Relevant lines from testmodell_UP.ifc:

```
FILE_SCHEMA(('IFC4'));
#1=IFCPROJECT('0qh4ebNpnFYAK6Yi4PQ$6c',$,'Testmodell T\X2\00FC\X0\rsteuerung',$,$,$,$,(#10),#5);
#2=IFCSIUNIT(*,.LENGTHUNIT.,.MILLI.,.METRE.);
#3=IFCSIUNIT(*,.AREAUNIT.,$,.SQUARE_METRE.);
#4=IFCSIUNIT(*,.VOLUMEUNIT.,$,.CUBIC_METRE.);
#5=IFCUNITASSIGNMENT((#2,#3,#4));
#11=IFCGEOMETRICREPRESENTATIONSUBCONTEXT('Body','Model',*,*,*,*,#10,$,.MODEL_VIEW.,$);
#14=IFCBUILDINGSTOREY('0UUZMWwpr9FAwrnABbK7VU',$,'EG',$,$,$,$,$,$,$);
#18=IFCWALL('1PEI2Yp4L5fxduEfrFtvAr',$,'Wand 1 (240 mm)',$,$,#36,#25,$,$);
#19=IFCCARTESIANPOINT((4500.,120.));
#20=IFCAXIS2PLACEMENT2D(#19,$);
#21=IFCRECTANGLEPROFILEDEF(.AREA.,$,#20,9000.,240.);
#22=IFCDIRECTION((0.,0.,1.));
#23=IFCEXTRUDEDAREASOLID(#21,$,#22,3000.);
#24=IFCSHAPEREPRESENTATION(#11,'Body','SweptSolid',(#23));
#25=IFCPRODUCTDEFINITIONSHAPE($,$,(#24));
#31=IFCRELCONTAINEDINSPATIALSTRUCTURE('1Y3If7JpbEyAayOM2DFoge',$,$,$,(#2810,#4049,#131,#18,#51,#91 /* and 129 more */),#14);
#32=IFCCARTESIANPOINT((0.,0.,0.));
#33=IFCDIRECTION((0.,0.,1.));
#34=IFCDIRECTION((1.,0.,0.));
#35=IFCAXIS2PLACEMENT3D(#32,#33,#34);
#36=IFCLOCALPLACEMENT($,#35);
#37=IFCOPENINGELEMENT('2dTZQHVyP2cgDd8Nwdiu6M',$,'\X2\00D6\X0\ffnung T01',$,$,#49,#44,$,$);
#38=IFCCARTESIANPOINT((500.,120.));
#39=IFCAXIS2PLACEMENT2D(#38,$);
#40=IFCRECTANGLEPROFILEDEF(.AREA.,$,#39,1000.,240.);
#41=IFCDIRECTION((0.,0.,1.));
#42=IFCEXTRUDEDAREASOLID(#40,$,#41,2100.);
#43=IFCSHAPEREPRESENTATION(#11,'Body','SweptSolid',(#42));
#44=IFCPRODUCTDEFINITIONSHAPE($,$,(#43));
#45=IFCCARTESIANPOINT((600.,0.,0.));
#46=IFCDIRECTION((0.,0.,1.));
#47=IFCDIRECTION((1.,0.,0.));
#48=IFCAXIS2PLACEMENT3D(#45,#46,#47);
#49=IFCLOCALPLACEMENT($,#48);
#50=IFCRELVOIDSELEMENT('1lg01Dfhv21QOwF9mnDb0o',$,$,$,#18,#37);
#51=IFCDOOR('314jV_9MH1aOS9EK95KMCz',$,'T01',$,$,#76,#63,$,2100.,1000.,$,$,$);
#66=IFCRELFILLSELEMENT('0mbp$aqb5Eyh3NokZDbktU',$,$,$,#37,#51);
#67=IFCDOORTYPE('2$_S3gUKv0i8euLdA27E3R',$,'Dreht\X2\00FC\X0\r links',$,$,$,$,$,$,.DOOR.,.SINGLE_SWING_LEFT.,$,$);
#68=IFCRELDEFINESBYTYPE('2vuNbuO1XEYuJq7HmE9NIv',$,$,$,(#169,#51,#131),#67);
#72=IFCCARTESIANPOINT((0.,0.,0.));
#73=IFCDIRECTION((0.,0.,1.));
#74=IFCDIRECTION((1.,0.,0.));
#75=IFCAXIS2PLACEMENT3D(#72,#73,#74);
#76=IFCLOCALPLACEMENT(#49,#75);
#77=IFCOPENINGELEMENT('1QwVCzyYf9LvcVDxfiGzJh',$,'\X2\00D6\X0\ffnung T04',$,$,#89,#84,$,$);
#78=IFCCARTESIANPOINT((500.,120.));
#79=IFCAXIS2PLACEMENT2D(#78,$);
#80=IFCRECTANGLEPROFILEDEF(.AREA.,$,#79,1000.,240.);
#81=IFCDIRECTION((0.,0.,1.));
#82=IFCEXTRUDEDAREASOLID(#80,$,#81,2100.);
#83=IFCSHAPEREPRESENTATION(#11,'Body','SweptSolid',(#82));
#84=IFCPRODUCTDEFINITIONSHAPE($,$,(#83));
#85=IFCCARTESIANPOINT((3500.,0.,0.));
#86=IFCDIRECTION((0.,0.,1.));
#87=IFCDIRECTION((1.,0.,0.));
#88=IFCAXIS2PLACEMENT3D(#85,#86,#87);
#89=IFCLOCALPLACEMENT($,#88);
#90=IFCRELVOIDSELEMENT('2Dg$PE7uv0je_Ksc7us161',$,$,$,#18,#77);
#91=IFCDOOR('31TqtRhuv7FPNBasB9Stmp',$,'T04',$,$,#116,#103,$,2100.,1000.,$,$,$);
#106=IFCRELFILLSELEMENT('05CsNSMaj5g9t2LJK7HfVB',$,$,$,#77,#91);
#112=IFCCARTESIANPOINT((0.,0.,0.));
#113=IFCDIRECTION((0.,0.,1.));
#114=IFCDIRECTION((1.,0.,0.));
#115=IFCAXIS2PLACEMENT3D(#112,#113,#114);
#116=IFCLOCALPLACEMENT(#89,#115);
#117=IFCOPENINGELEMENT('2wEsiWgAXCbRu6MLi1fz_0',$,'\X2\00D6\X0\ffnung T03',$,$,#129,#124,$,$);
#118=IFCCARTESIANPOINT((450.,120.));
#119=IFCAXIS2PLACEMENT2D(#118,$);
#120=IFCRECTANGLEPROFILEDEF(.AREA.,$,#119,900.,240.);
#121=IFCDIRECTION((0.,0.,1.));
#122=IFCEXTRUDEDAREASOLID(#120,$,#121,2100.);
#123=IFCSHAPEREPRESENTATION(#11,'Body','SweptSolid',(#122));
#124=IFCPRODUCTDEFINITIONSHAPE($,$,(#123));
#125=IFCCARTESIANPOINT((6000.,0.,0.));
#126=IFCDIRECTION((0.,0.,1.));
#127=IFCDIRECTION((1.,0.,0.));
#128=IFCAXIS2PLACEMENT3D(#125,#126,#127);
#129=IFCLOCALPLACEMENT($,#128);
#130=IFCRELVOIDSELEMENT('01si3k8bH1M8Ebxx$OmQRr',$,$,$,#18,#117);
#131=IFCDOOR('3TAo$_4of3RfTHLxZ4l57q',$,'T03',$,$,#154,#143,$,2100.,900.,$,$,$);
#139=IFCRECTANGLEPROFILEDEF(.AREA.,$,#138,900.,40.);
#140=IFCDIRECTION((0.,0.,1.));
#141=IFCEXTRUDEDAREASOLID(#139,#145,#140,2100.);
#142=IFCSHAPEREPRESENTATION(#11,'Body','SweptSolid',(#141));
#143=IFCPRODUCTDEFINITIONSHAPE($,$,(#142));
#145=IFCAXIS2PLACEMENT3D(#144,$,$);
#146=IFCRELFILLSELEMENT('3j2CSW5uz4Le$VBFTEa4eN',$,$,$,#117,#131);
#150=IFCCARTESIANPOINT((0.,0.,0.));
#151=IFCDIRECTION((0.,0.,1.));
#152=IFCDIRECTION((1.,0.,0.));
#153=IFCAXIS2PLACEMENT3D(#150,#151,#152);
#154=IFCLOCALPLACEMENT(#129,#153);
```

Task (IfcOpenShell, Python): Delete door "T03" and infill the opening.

```python
import ifcopenshell
import ifcopenshell.api.feature
import ifcopenshell.api.root
import ifcopenshell.geom
import ifcopenshell.util.shape

model = ifcopenshell.open("testmodell_UP.ifc")
settings = ifcopenshell.geom.settings()


def volume(element):
    """Net volume in cubic metres, openings subtracted."""
    shape = ifcopenshell.geom.create_shape(settings, element)
    return ifcopenshell.util.shape.get_volume(shape.geometry)


door = model.by_guid("3TAo$_4of3RfTHLxZ4l57q")
opening = door.FillsVoids[0].RelatingOpeningElement
wall = opening.VoidsElements[0].RelatingBuildingElement
before = volume(wall)

ifcopenshell.api.root.remove_product(model, product=door)
ifcopenshell.api.feature.remove_feature(model, feature=opening)

after = volume(wall)

print(f"wall volume {before:.3f} -> {after:.3f} m3")

model.write("testmodell_UP_rev.ifc")
```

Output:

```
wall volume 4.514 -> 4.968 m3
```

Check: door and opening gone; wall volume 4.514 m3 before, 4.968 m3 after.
